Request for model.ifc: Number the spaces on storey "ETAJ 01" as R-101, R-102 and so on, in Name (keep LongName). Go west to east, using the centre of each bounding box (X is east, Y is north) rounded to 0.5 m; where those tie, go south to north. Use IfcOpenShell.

First a look at what the model holds.

```python
import ifcopenshell
import ifcopenshell.util.element
import ifcopenshell.util.placement

model = ifcopenshell.open("model.ifc")
print(model.schema)
storey = next(s for s in model.by_type("IfcBuildingStorey") if s.Name == "ETAJ 01")
spaces = [e for e in ifcopenshell.util.element.get_decomposition(storey) if e.is_a("IfcSpace")]
for e in sorted(spaces, key=lambda e: e.id()):
    origin = ifcopenshell.util.placement.get_local_placement(e.ObjectPlacement)[:3, 3]
    print(e.id(), e.Name, e.LongName, origin.round(2) + 0.0, sep=" | ")
```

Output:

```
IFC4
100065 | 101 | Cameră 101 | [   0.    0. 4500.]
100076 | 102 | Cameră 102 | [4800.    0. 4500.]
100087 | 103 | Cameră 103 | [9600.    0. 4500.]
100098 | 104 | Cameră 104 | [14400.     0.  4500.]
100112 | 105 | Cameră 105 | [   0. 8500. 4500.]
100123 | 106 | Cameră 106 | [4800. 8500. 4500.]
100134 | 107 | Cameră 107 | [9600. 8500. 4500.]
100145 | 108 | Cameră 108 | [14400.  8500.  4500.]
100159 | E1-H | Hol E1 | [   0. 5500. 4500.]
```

```python
import ifcopenshell
import ifcopenshell.geom
import ifcopenshell.util.element
import ifcopenshell.util.shape

model = ifcopenshell.open("model.ifc")
settings = ifcopenshell.geom.settings()
settings.set("use-world-coords", True)


def centre(element):
    shape = ifcopenshell.geom.create_shape(settings, element)
    return ifcopenshell.util.shape.get_bbox_centroid(shape.geometry)


storey = next(s for s in model.by_type("IfcBuildingStorey") if s.Name == "ETAJ 01")
spaces = [e for e in ifcopenshell.util.element.get_decomposition(storey) if e.is_a("IfcSpace")]

# Insertion points can sit at a corner or the storey origin, so sort by the geometry (in metres).
centres = {e: centre(e) for e in spaces}
spaces.sort(key=lambda e: (round(centres[e][0] / 0.5), centres[e][1]))

for i, e in enumerate(spaces, start=1):
    number = f"R-1{i:02d}"
    e.Name = number
    print(e.id(), number)

model.write("model_v2.ifc")
```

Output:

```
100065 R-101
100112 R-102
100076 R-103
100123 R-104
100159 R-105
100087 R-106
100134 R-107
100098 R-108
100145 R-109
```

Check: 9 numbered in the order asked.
